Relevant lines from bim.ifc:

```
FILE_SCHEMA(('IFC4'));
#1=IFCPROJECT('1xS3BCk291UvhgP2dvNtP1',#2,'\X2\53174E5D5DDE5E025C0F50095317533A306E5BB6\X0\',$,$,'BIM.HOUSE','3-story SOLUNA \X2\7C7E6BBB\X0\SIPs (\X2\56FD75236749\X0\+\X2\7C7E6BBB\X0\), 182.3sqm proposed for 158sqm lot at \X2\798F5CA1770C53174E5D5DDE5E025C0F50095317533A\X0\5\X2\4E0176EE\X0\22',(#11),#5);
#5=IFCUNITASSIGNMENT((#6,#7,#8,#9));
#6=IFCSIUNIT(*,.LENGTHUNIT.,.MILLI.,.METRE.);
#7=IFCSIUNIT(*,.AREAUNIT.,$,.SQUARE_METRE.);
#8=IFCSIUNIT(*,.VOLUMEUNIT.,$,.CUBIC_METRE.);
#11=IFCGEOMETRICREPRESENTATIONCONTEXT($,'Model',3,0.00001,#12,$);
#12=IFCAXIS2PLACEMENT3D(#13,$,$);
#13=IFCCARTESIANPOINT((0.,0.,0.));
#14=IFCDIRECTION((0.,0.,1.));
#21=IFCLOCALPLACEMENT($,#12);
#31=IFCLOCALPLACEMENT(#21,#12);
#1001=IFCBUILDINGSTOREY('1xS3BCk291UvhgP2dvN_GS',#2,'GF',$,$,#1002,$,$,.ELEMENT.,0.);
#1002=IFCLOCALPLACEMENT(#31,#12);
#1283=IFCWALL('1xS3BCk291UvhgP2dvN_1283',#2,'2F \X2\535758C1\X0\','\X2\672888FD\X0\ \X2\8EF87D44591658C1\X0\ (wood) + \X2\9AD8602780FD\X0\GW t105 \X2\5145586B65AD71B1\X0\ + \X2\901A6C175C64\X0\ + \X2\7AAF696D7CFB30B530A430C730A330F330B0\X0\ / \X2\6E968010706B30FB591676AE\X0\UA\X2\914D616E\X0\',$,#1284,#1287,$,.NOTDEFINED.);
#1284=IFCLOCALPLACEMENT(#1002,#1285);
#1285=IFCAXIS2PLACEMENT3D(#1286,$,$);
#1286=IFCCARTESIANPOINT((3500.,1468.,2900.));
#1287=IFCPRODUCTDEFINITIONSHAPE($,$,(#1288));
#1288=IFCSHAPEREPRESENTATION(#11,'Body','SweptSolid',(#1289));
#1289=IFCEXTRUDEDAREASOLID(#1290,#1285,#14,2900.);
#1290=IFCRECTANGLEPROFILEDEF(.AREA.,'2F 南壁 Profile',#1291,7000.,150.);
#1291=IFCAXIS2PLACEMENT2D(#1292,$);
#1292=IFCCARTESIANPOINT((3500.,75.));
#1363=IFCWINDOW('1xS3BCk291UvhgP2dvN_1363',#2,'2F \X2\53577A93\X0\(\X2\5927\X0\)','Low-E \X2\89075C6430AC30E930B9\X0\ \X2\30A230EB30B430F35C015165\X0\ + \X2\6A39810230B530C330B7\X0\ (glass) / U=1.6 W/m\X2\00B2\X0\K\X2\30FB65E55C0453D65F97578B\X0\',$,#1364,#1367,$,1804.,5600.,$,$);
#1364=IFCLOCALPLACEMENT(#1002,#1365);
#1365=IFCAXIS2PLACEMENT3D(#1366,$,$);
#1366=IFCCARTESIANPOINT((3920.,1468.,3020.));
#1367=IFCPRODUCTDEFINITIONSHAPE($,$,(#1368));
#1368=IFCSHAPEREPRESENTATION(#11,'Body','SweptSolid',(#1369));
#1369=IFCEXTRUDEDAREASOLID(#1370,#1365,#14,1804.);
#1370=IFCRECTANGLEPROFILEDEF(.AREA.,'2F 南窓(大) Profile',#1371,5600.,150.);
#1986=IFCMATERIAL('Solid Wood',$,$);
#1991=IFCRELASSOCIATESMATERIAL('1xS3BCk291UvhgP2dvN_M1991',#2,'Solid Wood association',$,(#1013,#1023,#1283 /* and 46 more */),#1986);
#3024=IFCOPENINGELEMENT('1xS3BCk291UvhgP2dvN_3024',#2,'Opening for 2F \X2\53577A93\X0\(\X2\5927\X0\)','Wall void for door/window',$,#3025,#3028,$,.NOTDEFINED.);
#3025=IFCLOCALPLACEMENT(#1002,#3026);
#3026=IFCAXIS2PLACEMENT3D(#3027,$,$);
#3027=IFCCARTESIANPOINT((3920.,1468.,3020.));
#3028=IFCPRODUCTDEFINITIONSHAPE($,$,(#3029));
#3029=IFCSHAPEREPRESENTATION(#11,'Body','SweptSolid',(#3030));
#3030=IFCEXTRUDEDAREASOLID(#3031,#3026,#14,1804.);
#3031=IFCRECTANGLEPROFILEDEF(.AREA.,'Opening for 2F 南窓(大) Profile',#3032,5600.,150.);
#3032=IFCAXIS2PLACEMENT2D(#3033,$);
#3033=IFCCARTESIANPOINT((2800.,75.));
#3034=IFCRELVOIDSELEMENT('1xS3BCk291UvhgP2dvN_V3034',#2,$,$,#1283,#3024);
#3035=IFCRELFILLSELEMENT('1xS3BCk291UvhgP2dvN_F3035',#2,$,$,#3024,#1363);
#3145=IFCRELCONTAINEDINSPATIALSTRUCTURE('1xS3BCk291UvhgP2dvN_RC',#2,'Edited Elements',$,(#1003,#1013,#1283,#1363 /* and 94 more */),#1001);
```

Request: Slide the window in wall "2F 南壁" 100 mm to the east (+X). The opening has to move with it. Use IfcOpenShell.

```python
import ifcopenshell
import ifcopenshell.api.geometry
import ifcopenshell.util.placement
import ifcopenshell.util.unit

model = ifcopenshell.open("bim.ifc")
unit_scale = ifcopenshell.util.unit.calculate_unit_scale(model)

window = model.by_id(1363)
opening = window.FillsVoids[0].RelatingOpeningElement
wall = opening.VoidsElements[0].RelatingBuildingElement

wall_matrix = ifcopenshell.util.placement.get_local_placement(wall.ObjectPlacement)
shift = wall_matrix[:3, 0] * 0.1 / unit_scale
before = ifcopenshell.util.placement.get_local_placement(window.ObjectPlacement)[:3, 3].copy()

# The window is not placed relative to its opening, so move both.
for product in (opening, window):
    matrix = ifcopenshell.util.placement.get_local_placement(product.ObjectPlacement)
    matrix[:3, 3] += shift
    ifcopenshell.api.geometry.edit_object_placement(model, product=product, matrix=matrix, is_si=False)

after = ifcopenshell.util.placement.get_local_placement(window.ObjectPlacement)[:3, 3]
print("window moved by", (after - before).round(3) + 0.0)

model.write("bim_rev.ifc")
```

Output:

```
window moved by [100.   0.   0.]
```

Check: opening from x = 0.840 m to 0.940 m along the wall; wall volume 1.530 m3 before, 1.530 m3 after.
